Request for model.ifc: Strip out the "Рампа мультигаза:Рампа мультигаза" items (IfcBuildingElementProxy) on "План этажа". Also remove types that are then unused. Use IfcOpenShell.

First a look at what the model holds.

```python
import ifcopenshell
import ifcopenshell.util.element

model = ifcopenshell.open("model.ifc")
print(model.schema)
storey = next(s for s in model.by_type("IfcBuildingStorey") if s.Name == "План этажа")
proxies = [e for e in ifcopenshell.util.element.get_decomposition(storey) if e.is_a("IfcBuildingElementProxy")]
seen = {}
for e in proxies:
    element_type = ifcopenshell.util.element.get_type(e)
    name = element_type.Name if element_type not in (None, e) else None
    seen[name] = seen.get(name, 0) + 1
for name, count in sorted(seen.items(), key=str):
    print(count, "x", name)
```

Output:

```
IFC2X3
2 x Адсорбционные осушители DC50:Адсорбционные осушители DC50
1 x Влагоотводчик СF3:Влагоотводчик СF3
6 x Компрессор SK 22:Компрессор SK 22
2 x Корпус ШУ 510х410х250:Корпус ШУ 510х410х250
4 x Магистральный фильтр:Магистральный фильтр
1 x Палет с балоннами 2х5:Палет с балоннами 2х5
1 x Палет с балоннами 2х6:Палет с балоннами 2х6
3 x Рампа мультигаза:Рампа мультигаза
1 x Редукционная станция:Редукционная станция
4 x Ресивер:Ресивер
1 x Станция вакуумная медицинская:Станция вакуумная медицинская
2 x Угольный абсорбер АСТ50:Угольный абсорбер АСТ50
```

```python
import ifcopenshell
import ifcopenshell.api.root
import ifcopenshell.util.element

model = ifcopenshell.open("model.ifc")

storey = next(s for s in model.by_type("IfcBuildingStorey") if s.Name == "План этажа")
proxies = [e for e in ifcopenshell.util.element.get_decomposition(storey) if e.is_a("IfcBuildingElementProxy")]
targets = [e for e in proxies if (t := ifcopenshell.util.element.get_type(e)) not in (None, e) and t.Name == "Рампа мультигаза:Рампа мультигаза"]
types = {ifcopenshell.util.element.get_type(e) for e in targets} - {None, *targets}

for e in targets:
    ifcopenshell.api.root.remove_product(model, product=e)
print(len(targets), "removed")

unused = [t for t in types if not ifcopenshell.util.element.get_types(t)]
for t in unused:
    ifcopenshell.api.root.remove_product(model, product=t)
print(len(unused), "unused types removed")

model.write("model_edited.ifc")
```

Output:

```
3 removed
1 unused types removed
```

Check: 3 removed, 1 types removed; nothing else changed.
